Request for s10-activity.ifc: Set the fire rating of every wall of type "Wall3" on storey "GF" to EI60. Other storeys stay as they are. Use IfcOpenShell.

First a look at what the model holds.

```python
import ifcopenshell
import ifcopenshell.util.element

model = ifcopenshell.open("s10-activity.ifc")
print(model.schema)
storey = next(s for s in model.by_type("IfcBuildingStorey") if s.Name == "GF")
walls = [e for e in ifcopenshell.util.element.get_decomposition(storey) if e.is_a("IfcWall")]
seen = {}
for e in walls:
    element_type = ifcopenshell.util.element.get_type(e)
    key = (element_type.Name if element_type != e and element_type else None, ifcopenshell.util.element.get_pset(e, "Pset_WallCommon", "FireRating"))
    seen[key] = seen.get(key, 0) + 1
for (name, value), count in sorted(seen.items(), key=str):
    print(count, "x", name, "|", value)
```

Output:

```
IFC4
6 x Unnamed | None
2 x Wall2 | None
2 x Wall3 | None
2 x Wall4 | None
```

```python
import ifcopenshell
import ifcopenshell.api.pset
import ifcopenshell.util.element

model = ifcopenshell.open("s10-activity.ifc")

storey = next(s for s in model.by_type("IfcBuildingStorey") if s.Name == "GF")
walls = [e for e in ifcopenshell.util.element.get_decomposition(storey) if e.is_a("IfcWall")]

count = 0
for e in walls:
    element_type = ifcopenshell.util.element.get_type(e)
    if element_type in (None, e) or element_type.Name != "Wall3":
        continue
    # add_pset returns the element's existing set when there is one.
    pset = ifcopenshell.api.pset.add_pset(model, product=e, name="Pset_WallCommon")
    ifcopenshell.api.pset.edit_pset(model, pset=pset, properties={"FireRating": "EI60"})
    count += 1

print(count, "walls updated")

model.write("s10-activity_v2.ifc")
```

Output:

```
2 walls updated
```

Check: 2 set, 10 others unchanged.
